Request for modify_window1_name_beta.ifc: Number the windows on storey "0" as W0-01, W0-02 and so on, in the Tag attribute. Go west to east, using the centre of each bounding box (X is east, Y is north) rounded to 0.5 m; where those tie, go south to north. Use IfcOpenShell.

First a look at what the model holds.

```python
import ifcopenshell
import ifcopenshell.util.element
import ifcopenshell.util.placement

model = ifcopenshell.open("modify_window1_name_beta.ifc")
print(model.schema)
storey = next(s for s in model.by_type("IfcBuildingStorey") if s.Name == "0")
windows = [e for e in ifcopenshell.util.element.get_decomposition(storey) if e.is_a("IfcWindow")]
for e in sorted(windows, key=lambda e: e.id()):
    origin = ifcopenshell.util.placement.get_local_placement(e.ObjectPlacement)[:3, 3]
    print(e.id(), e.Tag, e.Name, origin.round(2) + 0.0, sep=" | ")
```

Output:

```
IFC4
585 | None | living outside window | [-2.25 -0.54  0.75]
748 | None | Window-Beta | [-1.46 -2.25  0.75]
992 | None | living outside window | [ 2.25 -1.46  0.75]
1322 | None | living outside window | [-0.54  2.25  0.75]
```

```python
import ifcopenshell
import ifcopenshell.geom
import ifcopenshell.util.element
import ifcopenshell.util.shape

model = ifcopenshell.open("modify_window1_name_beta.ifc")
settings = ifcopenshell.geom.settings()
settings.set("use-world-coords", True)


def centre(element):
    shape = ifcopenshell.geom.create_shape(settings, element)
    return ifcopenshell.util.shape.get_bbox_centroid(shape.geometry)


storey = next(s for s in model.by_type("IfcBuildingStorey") if s.Name == "0")
windows = [e for e in ifcopenshell.util.element.get_decomposition(storey) if e.is_a("IfcWindow")]

# Insertion points can sit at a corner or the storey origin, so sort by the geometry (in metres).
centres = {e: centre(e) for e in windows}
windows.sort(key=lambda e: (round(centres[e][0] / 0.5), centres[e][1]))

for i, e in enumerate(windows, start=1):
    number = f"W0-{i:02d}"
    e.Tag = number
    print(e.id(), number)

model.write("modify_window1_name_beta_v2.ifc")
```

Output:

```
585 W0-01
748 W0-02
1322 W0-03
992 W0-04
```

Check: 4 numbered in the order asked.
